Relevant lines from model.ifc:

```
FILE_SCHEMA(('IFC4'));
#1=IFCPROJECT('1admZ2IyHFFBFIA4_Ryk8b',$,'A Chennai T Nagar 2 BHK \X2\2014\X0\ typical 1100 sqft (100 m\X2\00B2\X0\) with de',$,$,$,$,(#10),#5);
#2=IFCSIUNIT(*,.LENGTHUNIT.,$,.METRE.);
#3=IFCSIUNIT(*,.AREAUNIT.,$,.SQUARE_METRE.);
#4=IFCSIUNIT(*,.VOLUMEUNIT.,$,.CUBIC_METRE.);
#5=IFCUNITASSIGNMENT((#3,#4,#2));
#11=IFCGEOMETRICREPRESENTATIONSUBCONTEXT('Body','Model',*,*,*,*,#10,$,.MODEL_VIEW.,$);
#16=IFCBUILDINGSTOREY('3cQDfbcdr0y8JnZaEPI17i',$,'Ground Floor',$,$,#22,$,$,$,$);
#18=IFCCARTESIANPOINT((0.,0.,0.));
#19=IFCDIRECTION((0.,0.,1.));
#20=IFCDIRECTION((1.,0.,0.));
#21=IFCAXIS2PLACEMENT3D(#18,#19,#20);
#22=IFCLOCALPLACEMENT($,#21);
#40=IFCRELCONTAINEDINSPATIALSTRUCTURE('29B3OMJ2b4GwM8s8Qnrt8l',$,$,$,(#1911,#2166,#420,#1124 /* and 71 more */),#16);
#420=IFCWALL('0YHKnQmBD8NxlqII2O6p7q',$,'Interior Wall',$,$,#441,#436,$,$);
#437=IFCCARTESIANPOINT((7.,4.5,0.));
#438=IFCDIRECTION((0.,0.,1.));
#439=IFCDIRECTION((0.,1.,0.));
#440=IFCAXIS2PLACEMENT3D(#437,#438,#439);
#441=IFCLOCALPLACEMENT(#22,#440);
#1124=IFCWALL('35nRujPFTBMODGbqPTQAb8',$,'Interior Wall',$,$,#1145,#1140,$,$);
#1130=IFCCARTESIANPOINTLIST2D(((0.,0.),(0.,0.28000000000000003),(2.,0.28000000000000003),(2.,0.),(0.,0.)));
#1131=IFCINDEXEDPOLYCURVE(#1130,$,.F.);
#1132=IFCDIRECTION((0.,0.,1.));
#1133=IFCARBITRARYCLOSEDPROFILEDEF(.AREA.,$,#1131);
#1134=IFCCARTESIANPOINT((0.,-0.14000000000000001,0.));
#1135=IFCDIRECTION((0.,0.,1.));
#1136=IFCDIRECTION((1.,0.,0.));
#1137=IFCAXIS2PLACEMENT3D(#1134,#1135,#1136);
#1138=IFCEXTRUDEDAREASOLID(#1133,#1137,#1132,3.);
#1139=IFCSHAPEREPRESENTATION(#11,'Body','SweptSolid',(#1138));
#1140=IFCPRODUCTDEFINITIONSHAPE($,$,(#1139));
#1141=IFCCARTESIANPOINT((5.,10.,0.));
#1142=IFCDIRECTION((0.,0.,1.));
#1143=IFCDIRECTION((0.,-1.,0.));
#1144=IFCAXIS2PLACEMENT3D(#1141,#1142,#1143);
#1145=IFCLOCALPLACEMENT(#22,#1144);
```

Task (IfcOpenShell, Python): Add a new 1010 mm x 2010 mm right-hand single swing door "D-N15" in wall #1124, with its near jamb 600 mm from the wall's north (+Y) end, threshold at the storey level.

```python
import numpy as np
import ifcopenshell
import ifcopenshell.api.feature
import ifcopenshell.api.geometry
import ifcopenshell.api.root
import ifcopenshell.api.spatial
import ifcopenshell.geom
import ifcopenshell.util.element
import ifcopenshell.util.placement
import ifcopenshell.util.representation
import ifcopenshell.util.shape
import ifcopenshell.util.unit

model = ifcopenshell.open("model.ifc")
unit_scale = ifcopenshell.util.unit.calculate_unit_scale(model)
settings = ifcopenshell.geom.settings()


def volume(element):
    """Net volume in cubic metres, openings subtracted."""
    shape = ifcopenshell.geom.create_shape(settings, element)
    return ifcopenshell.util.shape.get_volume(shape.geometry)


wall = model.by_guid("35nRujPFTBMODGbqPTQAb8")
storey = ifcopenshell.util.element.get_container(wall, ifc_class="IfcBuildingStorey")
context = ifcopenshell.util.representation.get_context(model, "Model", "Body", "MODEL_VIEW")
before = volume(wall)

width, height, from_end, sill = 1.01, 2.01, 0.6, 0.0  # metres

# The wall runs along its own X axis, and the end named is its -X end.
wall_shape = ifcopenshell.geom.create_shape(settings, wall)
x, y, z = ifcopenshell.util.shape.get_vertices(wall_shape.geometry).T
start = x.min() + from_end
face, thickness = float(y.min()), float(y.max() - y.min())
wall_matrix = ifcopenshell.util.placement.get_local_placement(wall.ObjectPlacement)
level = ifcopenshell.util.placement.get_local_placement(storey.ObjectPlacement)[2, 3]


def in_wall(x, y):
    """Placement at x, y metres in the wall's axes, at sill height."""
    matrix = wall_matrix.copy()
    matrix[:, 3] = wall_matrix @ np.array([x / unit_scale, y / unit_scale, 0.0, 1.0])
    matrix[2, 3] = level + sill / unit_scale
    return matrix


# Opening: a box that overshoots both wall faces by 50 mm.
opening = ifcopenshell.api.root.create_entity(model, ifc_class="IfcOpeningElement", predefined_type="OPENING")
box = ifcopenshell.api.geometry.add_wall_representation(
    model, context=context, length=width, height=height, thickness=thickness + 0.1
)
ifcopenshell.api.geometry.assign_representation(model, product=opening, representation=box)
ifcopenshell.api.geometry.edit_object_placement(model, product=opening, matrix=in_wall(start, face - 0.05), is_si=False)
ifcopenshell.api.feature.add_feature(model, feature=opening, element=wall)

door = ifcopenshell.api.root.create_entity(model, ifc_class="IfcDoor", name="D-N15", predefined_type="DOOR")
door.OverallWidth, door.OverallHeight = width / unit_scale, height / unit_scale
door.OperationType = "SINGLE_SWING_RIGHT"
body = ifcopenshell.api.geometry.add_door_representation(
    model,
    context=context,
    overall_width=door.OverallWidth,
    overall_height=door.OverallHeight,
    operation_type="SINGLE_SWING_RIGHT",
    lining_properties={"LiningDepth": thickness / unit_scale, "ThresholdDepth": thickness / unit_scale},
)
ifcopenshell.api.geometry.assign_representation(model, product=door, representation=body)
ifcopenshell.api.spatial.assign_container(model, products=[door], relating_structure=storey)
ifcopenshell.api.feature.add_filling(model, opening=opening, element=door)

# The lining spans the wall, so the door starts at the wall face.
ifcopenshell.api.geometry.edit_object_placement(model, product=door, matrix=in_wall(start, face), is_si=False)

after = volume(wall)

print(f"wall volume {before:.3f} -> {after:.3f} m3")

model.write("model_edited.ifc")
```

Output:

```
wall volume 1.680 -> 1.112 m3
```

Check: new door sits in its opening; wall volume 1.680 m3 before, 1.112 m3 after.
